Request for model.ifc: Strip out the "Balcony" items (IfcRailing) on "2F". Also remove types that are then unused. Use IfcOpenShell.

First a look at what the model holds.

```python
import ifcopenshell
import ifcopenshell.util.element

model = ifcopenshell.open("model.ifc")
print(model.schema)
storey = next(s for s in model.by_type("IfcBuildingStorey") if s.Name == "2F")
railings = [e for e in ifcopenshell.util.element.get_decomposition(storey) if e.is_a("IfcRailing")]
seen = {}
for e in railings:
    element_type = ifcopenshell.util.element.get_type(e)
    name = element_type.Name if element_type not in (None, e) else None
    seen[name] = seen.get(name, 0) + 1
for name, count in sorted(seen.items(), key=str):
    print(count, "x", name)
```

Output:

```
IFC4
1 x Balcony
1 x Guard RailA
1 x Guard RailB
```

```python
import ifcopenshell
import ifcopenshell.api.root
import ifcopenshell.util.element

model = ifcopenshell.open("model.ifc")

storey = next(s for s in model.by_type("IfcBuildingStorey") if s.Name == "2F")
railings = [e for e in ifcopenshell.util.element.get_decomposition(storey) if e.is_a("IfcRailing")]
targets = [e for e in railings if (t := ifcopenshell.util.element.get_type(e)) not in (None, e) and t.Name == "Balcony"]
types = {ifcopenshell.util.element.get_type(e) for e in targets} - {None, *targets}

for e in targets:
    ifcopenshell.api.root.remove_product(model, product=e)
print(len(targets), "removed")

unused = [t for t in types if not ifcopenshell.util.element.get_types(t)]
for t in unused:
    ifcopenshell.api.root.remove_product(model, product=t)
print(len(unused), "unused types removed")

model.write("model_updated.ifc")
```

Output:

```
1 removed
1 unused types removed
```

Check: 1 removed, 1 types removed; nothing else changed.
